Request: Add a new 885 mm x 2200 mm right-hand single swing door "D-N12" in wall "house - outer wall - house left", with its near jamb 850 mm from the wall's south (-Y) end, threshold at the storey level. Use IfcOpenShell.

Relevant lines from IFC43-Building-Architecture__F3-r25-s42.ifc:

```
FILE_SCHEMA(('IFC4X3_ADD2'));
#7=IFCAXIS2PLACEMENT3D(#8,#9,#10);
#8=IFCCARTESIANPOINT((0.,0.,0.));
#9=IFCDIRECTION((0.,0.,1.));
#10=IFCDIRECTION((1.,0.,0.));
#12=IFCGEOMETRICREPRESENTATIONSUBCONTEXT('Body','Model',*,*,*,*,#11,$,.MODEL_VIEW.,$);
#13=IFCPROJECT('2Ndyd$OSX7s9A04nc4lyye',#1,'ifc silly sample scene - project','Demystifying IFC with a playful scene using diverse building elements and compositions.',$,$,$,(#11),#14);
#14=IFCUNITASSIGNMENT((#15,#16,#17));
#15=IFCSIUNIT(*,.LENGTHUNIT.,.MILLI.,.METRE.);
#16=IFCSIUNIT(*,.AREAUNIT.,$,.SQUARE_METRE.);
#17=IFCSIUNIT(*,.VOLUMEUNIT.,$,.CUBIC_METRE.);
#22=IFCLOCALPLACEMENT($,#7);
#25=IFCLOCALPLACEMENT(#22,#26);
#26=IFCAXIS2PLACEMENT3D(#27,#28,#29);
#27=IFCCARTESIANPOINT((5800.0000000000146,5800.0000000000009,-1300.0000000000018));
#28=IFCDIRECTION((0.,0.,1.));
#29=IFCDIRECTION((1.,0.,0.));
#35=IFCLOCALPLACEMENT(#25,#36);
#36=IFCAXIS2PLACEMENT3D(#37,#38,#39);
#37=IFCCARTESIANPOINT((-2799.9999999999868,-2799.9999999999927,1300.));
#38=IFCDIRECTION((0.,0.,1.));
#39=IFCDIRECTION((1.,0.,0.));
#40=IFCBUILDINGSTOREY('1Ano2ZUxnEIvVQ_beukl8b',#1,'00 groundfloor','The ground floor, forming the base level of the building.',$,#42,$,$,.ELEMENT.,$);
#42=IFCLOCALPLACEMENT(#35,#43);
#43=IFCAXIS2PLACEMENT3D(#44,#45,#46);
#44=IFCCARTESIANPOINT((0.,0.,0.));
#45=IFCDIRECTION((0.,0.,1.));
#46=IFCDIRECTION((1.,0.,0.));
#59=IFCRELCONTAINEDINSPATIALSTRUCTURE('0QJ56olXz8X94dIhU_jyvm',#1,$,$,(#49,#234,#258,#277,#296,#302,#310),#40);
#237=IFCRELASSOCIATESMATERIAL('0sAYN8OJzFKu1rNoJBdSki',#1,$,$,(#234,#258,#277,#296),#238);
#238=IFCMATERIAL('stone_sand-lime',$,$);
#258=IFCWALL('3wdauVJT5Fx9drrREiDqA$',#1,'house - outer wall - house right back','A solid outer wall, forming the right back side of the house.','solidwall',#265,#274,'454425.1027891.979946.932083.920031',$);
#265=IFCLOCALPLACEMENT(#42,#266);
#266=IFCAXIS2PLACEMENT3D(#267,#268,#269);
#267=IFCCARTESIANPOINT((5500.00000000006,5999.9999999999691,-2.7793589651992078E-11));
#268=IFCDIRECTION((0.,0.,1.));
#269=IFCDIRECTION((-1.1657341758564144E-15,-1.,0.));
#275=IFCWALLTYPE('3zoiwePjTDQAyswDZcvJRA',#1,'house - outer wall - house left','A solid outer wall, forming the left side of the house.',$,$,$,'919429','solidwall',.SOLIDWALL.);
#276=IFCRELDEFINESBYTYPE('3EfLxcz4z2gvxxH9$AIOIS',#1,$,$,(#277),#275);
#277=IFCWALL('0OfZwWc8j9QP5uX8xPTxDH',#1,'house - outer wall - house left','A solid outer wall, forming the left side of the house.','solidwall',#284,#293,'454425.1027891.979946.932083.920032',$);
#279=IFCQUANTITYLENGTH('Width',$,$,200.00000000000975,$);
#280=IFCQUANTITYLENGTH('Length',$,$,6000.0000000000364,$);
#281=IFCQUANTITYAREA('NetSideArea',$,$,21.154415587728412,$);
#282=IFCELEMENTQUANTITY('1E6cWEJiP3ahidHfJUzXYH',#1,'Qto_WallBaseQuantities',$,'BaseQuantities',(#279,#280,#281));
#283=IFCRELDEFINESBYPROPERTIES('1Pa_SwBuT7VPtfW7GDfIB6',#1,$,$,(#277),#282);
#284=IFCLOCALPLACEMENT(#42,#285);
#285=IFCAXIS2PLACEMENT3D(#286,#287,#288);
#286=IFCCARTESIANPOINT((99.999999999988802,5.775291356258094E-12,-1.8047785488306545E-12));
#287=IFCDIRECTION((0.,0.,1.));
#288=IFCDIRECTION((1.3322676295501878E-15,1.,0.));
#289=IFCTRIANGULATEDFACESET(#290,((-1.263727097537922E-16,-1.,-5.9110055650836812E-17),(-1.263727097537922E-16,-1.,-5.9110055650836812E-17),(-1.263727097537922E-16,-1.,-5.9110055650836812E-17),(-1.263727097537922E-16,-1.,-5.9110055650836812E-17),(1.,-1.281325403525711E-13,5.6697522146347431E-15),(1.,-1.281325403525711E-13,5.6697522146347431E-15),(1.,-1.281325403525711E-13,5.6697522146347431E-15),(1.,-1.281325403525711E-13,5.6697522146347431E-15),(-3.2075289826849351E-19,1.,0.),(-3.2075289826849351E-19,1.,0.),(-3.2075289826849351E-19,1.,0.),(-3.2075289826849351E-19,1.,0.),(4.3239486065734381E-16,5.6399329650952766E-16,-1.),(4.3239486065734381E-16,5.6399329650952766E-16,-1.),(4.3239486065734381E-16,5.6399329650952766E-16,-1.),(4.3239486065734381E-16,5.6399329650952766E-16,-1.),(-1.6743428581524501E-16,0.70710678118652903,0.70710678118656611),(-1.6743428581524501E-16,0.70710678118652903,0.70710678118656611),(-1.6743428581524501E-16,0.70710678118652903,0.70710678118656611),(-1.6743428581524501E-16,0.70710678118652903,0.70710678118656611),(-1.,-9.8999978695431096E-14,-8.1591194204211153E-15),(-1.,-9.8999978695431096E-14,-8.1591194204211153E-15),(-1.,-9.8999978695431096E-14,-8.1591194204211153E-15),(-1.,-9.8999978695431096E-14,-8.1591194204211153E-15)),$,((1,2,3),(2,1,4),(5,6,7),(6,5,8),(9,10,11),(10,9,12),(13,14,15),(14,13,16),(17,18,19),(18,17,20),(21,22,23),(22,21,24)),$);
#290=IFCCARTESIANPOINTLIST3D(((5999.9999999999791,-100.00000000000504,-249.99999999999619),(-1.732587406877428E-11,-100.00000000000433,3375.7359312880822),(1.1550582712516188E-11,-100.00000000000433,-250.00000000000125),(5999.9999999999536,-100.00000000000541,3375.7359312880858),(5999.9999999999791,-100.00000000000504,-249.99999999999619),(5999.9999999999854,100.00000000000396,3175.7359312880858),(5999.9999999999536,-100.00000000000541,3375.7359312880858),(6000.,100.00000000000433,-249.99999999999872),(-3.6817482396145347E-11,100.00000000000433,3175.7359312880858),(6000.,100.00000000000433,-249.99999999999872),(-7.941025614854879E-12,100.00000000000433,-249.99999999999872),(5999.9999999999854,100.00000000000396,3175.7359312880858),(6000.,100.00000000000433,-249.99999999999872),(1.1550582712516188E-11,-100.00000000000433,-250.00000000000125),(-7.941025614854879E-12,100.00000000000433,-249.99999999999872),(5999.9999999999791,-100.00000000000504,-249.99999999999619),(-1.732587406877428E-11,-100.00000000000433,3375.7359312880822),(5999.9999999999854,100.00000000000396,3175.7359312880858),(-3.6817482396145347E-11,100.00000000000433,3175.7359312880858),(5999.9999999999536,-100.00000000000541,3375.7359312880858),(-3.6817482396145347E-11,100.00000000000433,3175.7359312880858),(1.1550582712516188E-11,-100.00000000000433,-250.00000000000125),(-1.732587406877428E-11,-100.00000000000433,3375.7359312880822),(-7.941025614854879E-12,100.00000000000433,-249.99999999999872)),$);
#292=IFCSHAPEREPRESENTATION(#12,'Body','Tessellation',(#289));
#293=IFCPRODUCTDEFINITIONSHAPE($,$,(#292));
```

```python
import numpy as np
import ifcopenshell
import ifcopenshell.api.feature
import ifcopenshell.api.geometry
import ifcopenshell.api.pset
import ifcopenshell.api.root
import ifcopenshell.api.spatial
import ifcopenshell.geom
import ifcopenshell.util.element
import ifcopenshell.util.placement
import ifcopenshell.util.representation
import ifcopenshell.util.shape
import ifcopenshell.util.unit

model = ifcopenshell.open("IFC43-Building-Architecture__F3-r25-s42.ifc")
unit_scale = ifcopenshell.util.unit.calculate_unit_scale(model)
area_scale = ifcopenshell.util.unit.calculate_unit_scale(model, "AREAUNIT")
settings = ifcopenshell.geom.settings()


def volume(element):
    """Net volume in cubic metres, openings subtracted."""
    shape = ifcopenshell.geom.create_shape(settings, element)
    return ifcopenshell.util.shape.get_volume(shape.geometry)


wall = model.by_guid("0OfZwWc8j9QP5uX8xPTxDH")
storey = ifcopenshell.util.element.get_container(wall, ifc_class="IfcBuildingStorey")
context = ifcopenshell.util.representation.get_context(model, "Model", "Body", "MODEL_VIEW")
before = volume(wall)

width, height, from_end, sill = 0.885, 2.2, 0.85, 0.0  # metres

# The wall runs along its own X axis, and the end named is its -X end.
wall_shape = ifcopenshell.geom.create_shape(settings, wall)
x, y, z = ifcopenshell.util.shape.get_vertices(wall_shape.geometry).T
start = x.min() + from_end
face, thickness = float(y.min()), float(y.max() - y.min())
wall_matrix = ifcopenshell.util.placement.get_local_placement(wall.ObjectPlacement)
level = ifcopenshell.util.placement.get_local_placement(storey.ObjectPlacement)[2, 3]


def in_wall(x, y):
    """Placement at x, y metres in the wall's axes, at sill height."""
    matrix = wall_matrix.copy()
    matrix[:, 3] = wall_matrix @ np.array([x / unit_scale, y / unit_scale, 0.0, 1.0])
    matrix[2, 3] = level + sill / unit_scale
    return matrix


# Opening: a box that overshoots both wall faces by 50 mm.
opening = ifcopenshell.api.root.create_entity(model, ifc_class="IfcOpeningElement", predefined_type="OPENING")
box = ifcopenshell.api.geometry.add_wall_representation(
    model, context=context, length=width, height=height, thickness=thickness + 0.1
)
ifcopenshell.api.geometry.assign_representation(model, product=opening, representation=box)
ifcopenshell.api.geometry.edit_object_placement(model, product=opening, matrix=in_wall(start, face - 0.05), is_si=False)
ifcopenshell.api.feature.add_feature(model, feature=opening, element=wall)

door = ifcopenshell.api.root.create_entity(model, ifc_class="IfcDoor", name="D-N12", predefined_type="DOOR")
door.OverallWidth, door.OverallHeight = width / unit_scale, height / unit_scale
door.OperationType = "SINGLE_SWING_RIGHT"
body = ifcopenshell.api.geometry.add_door_representation(
    model,
    context=context,
    overall_width=door.OverallWidth,
    overall_height=door.OverallHeight,
    operation_type="SINGLE_SWING_RIGHT",
    lining_properties={"LiningDepth": thickness / unit_scale, "ThresholdDepth": thickness / unit_scale},
)
ifcopenshell.api.geometry.assign_representation(model, product=door, representation=body)
ifcopenshell.api.spatial.assign_container(model, products=[door], relating_structure=storey)
ifcopenshell.api.feature.add_filling(model, opening=opening, element=door)

# The lining spans the wall, so the door starts at the wall face.
ifcopenshell.api.geometry.edit_object_placement(model, product=door, matrix=in_wall(start, face), is_si=False)

after = volume(wall)

# Update the wall's stored quantities.
qto = model.by_id(ifcopenshell.util.element.get_pset(wall, "Qto_WallBaseQuantities", should_inherit=False)["id"])
ifcopenshell.api.pset.edit_qto(model, qto=qto, properties={"NetSideArea": after / thickness / area_scale})

print(f"wall volume {before:.3f} -> {after:.3f} m3")

model.write("IFC43-Building-Architecture__F3-r25-s42-out.ifc")
```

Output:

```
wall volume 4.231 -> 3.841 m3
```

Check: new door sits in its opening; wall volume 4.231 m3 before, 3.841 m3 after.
